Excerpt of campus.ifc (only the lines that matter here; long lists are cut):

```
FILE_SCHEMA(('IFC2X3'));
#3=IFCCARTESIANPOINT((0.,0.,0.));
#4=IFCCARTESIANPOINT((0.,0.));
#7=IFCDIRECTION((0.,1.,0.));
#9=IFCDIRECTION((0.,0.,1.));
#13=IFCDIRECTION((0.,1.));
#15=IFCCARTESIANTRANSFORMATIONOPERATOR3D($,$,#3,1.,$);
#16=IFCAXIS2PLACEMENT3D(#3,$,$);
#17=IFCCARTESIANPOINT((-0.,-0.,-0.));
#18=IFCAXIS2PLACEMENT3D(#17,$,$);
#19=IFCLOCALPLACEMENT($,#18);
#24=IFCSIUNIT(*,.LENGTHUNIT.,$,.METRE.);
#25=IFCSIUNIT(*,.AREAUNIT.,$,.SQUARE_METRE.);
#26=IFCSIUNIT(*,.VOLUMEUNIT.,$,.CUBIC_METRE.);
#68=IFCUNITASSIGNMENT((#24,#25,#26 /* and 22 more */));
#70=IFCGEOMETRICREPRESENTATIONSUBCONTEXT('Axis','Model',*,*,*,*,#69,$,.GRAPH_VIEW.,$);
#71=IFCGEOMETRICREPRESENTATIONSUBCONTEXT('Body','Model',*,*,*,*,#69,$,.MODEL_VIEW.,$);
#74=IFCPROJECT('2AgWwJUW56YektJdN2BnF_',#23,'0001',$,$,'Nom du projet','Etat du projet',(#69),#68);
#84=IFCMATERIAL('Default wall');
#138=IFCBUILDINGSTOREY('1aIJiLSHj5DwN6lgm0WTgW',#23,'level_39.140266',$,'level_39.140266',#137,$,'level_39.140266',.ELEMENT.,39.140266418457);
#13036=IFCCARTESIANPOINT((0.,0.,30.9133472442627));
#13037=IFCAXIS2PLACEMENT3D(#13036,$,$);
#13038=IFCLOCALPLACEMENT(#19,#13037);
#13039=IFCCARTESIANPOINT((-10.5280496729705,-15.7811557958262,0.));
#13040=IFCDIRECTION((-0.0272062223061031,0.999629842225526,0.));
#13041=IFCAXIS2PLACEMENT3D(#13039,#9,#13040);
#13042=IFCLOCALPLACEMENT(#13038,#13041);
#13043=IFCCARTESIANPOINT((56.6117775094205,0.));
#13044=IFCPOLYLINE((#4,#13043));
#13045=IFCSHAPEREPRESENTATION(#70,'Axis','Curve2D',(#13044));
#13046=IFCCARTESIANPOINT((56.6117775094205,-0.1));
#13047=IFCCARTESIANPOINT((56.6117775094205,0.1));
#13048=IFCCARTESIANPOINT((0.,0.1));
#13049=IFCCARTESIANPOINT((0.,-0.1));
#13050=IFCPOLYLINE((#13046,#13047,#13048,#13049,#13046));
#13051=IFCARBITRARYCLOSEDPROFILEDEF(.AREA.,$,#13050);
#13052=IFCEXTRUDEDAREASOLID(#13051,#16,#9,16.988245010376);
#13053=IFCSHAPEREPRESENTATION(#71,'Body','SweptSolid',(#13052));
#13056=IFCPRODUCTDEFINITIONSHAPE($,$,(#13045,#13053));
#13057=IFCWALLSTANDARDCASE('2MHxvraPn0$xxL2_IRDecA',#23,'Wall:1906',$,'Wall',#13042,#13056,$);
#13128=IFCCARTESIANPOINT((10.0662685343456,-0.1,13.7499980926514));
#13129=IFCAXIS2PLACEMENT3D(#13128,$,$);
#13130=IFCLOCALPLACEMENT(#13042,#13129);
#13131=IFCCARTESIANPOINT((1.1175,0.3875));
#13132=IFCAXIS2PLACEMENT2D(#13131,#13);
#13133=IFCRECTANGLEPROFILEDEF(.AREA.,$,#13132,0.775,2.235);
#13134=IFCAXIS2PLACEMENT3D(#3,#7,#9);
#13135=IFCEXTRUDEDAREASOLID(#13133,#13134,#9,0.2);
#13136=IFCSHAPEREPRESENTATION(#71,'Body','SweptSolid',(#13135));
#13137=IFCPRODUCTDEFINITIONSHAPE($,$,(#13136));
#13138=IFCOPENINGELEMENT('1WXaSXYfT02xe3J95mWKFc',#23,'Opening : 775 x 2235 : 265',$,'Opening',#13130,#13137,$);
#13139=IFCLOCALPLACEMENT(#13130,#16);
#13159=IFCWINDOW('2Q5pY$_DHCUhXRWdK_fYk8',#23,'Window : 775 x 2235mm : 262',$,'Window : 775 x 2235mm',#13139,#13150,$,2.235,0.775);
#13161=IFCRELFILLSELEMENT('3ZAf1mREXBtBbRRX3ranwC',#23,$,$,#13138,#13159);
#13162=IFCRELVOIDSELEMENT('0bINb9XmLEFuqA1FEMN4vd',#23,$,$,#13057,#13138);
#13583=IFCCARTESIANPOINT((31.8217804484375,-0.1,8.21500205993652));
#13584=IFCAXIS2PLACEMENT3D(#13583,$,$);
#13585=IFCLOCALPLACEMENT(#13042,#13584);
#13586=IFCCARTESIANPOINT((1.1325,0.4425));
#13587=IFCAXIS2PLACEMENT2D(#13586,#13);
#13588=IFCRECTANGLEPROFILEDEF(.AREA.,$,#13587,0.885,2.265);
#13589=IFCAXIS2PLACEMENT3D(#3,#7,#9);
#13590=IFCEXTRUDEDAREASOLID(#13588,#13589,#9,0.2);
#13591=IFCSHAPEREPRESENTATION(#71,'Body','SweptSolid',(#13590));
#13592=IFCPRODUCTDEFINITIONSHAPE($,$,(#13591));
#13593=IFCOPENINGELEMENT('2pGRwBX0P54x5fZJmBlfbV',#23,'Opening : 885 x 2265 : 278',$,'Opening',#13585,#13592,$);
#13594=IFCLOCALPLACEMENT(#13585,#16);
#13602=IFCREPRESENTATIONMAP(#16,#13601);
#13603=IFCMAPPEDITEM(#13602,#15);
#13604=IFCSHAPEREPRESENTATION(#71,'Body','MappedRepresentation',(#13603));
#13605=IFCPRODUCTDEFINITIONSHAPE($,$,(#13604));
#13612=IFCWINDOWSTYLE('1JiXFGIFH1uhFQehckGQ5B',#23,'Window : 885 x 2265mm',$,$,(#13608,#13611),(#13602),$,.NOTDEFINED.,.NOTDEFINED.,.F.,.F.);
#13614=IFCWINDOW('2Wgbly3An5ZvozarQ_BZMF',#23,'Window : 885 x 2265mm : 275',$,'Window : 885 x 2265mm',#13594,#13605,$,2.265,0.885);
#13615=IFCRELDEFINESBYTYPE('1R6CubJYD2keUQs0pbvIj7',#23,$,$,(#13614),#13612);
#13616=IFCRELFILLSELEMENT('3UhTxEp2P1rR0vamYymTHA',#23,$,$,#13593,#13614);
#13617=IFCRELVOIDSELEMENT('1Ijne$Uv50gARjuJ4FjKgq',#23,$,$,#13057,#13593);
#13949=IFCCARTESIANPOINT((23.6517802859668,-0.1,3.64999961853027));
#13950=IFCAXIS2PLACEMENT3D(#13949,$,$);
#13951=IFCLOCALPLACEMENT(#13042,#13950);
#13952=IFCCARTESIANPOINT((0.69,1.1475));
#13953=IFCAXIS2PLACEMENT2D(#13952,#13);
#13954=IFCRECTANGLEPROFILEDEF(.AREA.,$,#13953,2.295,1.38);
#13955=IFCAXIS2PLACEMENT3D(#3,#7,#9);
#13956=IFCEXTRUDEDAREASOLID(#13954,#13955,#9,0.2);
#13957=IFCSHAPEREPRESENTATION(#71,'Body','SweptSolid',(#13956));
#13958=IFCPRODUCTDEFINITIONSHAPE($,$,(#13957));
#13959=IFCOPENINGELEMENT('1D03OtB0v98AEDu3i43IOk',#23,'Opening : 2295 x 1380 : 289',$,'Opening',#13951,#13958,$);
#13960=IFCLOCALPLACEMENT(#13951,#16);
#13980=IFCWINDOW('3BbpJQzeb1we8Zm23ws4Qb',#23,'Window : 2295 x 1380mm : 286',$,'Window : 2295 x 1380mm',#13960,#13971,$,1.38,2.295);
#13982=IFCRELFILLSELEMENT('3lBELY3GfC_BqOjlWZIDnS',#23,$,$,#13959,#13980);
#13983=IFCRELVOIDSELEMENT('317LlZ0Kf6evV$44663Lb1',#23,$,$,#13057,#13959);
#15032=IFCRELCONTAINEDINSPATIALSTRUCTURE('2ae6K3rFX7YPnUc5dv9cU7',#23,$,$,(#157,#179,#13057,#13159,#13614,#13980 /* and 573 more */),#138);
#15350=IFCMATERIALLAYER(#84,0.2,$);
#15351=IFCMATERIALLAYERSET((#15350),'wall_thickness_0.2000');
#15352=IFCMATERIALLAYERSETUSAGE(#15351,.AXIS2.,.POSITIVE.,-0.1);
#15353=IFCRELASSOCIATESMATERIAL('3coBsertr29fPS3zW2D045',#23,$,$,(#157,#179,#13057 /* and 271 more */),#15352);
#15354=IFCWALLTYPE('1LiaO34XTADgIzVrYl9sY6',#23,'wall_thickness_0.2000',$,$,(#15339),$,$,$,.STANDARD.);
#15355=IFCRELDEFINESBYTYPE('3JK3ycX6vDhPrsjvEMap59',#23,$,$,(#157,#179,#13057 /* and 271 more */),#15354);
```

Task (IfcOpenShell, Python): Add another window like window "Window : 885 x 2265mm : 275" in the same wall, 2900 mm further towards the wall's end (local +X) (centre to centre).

```python
import ifcopenshell
import ifcopenshell.api.feature
import ifcopenshell.api.geometry
import ifcopenshell.api.root
import ifcopenshell.geom
import ifcopenshell.util.element
import ifcopenshell.util.placement
import ifcopenshell.util.shape

model = ifcopenshell.open("campus.ifc")
settings = ifcopenshell.geom.settings()


def volume(element):
    """Net volume in cubic metres, openings subtracted."""
    shape = ifcopenshell.geom.create_shape(settings, element)
    return ifcopenshell.util.shape.get_volume(shape.geometry)


window = model.by_id(13614)
opening = window.FillsVoids[0].RelatingOpeningElement
wall = opening.VoidsElements[0].RelatingBuildingElement
before = volume(wall)
shift = ifcopenshell.util.placement.get_local_placement(wall.ObjectPlacement)[:3, 0] * 2.9

# copy_class copies the void relationship, type, container and properties, but no geometry.
new_opening = ifcopenshell.api.root.copy_class(model, product=opening)
new_opening.Representation = ifcopenshell.util.element.copy_deep(
    model, opening.Representation, exclude=["IfcGeometricRepresentationContext", "IfcRepresentationMap"]
)
new_opening.Name = "Opening : 885 x 2265"
new_window = ifcopenshell.api.root.copy_class(model, product=window)
new_window.Representation = ifcopenshell.util.element.copy_deep(
    model, window.Representation, exclude=["IfcGeometricRepresentationContext", "IfcRepresentationMap"]
)
new_window.Name = "Window : 885 x 2265mm"
fills = ifcopenshell.api.feature.add_filling(model, opening=new_opening, element=new_window)
fills.OwnerHistory = new_window.OwnerHistory  # required in IFC2X3

for old, new in ((opening, new_opening), (window, new_window)):
    matrix = ifcopenshell.util.placement.get_local_placement(old.ObjectPlacement)
    matrix[:3, 3] += shift
    ifcopenshell.api.geometry.edit_object_placement(model, product=new, matrix=matrix, is_si=False)

after = volume(wall)

print(f"wall volume {before:.3f} -> {after:.3f} m3")

model.write("campus_edited.ifc")
```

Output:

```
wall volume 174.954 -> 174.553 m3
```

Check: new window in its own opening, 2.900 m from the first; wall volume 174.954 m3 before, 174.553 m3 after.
